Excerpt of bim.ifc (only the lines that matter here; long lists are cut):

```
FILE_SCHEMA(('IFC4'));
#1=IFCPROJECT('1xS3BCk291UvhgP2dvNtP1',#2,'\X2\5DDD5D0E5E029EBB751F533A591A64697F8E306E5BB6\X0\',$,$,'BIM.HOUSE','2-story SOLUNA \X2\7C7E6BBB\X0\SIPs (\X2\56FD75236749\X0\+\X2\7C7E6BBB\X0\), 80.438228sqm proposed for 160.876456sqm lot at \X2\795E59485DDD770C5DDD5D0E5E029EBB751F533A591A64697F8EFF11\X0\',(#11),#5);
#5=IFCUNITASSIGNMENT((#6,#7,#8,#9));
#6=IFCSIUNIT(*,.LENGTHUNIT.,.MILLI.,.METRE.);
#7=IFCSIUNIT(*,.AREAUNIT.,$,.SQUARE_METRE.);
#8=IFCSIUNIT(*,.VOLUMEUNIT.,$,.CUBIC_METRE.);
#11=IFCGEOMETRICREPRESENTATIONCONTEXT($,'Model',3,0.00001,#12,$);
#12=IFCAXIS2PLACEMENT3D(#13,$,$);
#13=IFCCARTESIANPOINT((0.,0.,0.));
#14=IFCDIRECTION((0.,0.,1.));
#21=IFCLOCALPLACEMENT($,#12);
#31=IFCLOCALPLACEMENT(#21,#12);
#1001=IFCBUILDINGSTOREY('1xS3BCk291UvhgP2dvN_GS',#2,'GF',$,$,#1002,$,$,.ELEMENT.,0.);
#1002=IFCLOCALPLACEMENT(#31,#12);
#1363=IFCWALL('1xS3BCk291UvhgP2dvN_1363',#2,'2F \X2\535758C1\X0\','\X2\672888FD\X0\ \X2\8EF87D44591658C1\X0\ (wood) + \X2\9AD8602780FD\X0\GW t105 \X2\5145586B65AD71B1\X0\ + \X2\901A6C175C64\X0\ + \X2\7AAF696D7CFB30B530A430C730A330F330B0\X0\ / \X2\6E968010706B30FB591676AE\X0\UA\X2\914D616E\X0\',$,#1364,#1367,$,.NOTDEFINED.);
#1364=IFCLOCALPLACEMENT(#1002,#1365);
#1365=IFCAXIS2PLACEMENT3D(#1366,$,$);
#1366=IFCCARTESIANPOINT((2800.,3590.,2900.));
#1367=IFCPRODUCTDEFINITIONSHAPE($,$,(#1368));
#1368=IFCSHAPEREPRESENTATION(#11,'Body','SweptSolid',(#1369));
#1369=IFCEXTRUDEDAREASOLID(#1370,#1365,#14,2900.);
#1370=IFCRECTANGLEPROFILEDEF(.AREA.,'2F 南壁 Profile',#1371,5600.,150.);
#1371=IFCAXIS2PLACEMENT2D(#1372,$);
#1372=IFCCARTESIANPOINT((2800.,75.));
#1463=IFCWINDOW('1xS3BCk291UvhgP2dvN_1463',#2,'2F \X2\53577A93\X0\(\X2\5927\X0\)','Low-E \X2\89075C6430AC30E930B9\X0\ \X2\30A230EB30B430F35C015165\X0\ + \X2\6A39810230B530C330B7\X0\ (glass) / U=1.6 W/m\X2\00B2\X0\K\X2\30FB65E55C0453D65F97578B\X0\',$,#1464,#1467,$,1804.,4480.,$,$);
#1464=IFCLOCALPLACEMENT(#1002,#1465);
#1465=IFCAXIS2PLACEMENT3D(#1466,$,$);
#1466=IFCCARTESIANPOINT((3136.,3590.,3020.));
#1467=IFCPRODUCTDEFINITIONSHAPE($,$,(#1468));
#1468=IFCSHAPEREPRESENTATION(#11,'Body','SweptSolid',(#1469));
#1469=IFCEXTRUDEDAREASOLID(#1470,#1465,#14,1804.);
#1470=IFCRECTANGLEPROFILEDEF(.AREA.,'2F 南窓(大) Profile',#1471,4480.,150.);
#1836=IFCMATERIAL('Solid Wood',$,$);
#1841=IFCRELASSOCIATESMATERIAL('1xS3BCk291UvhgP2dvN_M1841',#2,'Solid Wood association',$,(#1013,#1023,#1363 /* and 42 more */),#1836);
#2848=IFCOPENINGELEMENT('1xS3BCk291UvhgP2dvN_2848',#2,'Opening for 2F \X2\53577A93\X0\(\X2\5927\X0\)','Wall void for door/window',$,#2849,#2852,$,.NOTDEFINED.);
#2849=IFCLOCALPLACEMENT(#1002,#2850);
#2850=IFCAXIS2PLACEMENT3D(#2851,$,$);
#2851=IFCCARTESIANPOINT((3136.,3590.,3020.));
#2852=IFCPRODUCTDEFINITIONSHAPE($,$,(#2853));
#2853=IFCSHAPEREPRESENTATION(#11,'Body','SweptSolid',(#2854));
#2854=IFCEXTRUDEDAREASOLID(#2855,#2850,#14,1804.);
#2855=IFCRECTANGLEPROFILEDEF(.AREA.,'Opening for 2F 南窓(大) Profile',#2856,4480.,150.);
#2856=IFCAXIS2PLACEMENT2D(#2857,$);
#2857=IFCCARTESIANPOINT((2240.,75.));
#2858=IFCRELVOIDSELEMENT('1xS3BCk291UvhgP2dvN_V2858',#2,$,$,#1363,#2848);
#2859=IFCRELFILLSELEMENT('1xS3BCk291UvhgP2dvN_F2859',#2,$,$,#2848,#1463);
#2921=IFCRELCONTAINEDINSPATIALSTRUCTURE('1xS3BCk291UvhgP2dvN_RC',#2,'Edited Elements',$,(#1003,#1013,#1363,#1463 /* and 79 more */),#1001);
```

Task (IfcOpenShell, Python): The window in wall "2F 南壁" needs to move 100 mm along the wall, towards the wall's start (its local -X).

```python
import ifcopenshell
import ifcopenshell.api.geometry
import ifcopenshell.util.placement
import ifcopenshell.util.unit

model = ifcopenshell.open("bim.ifc")
unit_scale = ifcopenshell.util.unit.calculate_unit_scale(model)

window = model.by_guid("1xS3BCk291UvhgP2dvN_1463")
opening = window.FillsVoids[0].RelatingOpeningElement
wall = opening.VoidsElements[0].RelatingBuildingElement

wall_matrix = ifcopenshell.util.placement.get_local_placement(wall.ObjectPlacement)
shift = wall_matrix[:3, 0] * -0.1 / unit_scale
before = ifcopenshell.util.placement.get_local_placement(window.ObjectPlacement)[:3, 3].copy()

# The window is not placed relative to its opening, so move both.
for product in (opening, window):
    matrix = ifcopenshell.util.placement.get_local_placement(product.ObjectPlacement)
    matrix[:3, 3] += shift
    ifcopenshell.api.geometry.edit_object_placement(model, product=product, matrix=matrix, is_si=False)

after = ifcopenshell.util.placement.get_local_placement(window.ObjectPlacement)[:3, 3]
print("window moved by", (after - before).round(3) + 0.0)

model.write("bim_v2.ifc")
```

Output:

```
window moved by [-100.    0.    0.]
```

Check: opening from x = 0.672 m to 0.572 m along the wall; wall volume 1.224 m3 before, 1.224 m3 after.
